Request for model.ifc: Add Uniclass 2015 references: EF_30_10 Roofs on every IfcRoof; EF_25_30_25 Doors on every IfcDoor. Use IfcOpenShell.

First a look at what the model holds.

```python
import ifcopenshell

model = ifcopenshell.open("model.ifc")
print(model.schema)
print("classifications:", [c.Name for c in model.by_type("IfcClassification")])
for ifc_class in ("IfcDoor", "IfcRoof", "IfcStair", "IfcWall", "IfcWindow"):
    print(ifc_class, len(model.by_type(ifc_class)))
```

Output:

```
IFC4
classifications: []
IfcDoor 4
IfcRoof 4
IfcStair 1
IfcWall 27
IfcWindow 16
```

```python
import ifcopenshell
import ifcopenshell.api.classification

model = ifcopenshell.open("model.ifc")

system = ifcopenshell.api.classification.add_classification(model, classification="Uniclass 2015")

codes = {
    "IfcRoof": ("EF_30_10", "Roofs"),
    "IfcDoor": ("EF_25_30_25", "Doors"),
}
for ifc_class, (code, name) in codes.items():
    products = model.by_type(ifc_class)
    ifcopenshell.api.classification.add_reference(
        model, products=products, classification=system, identification=code, name=name
    )
    print(code, len(products))

model.write("model-out.ifc")
```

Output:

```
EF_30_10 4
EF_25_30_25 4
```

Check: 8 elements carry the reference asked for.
